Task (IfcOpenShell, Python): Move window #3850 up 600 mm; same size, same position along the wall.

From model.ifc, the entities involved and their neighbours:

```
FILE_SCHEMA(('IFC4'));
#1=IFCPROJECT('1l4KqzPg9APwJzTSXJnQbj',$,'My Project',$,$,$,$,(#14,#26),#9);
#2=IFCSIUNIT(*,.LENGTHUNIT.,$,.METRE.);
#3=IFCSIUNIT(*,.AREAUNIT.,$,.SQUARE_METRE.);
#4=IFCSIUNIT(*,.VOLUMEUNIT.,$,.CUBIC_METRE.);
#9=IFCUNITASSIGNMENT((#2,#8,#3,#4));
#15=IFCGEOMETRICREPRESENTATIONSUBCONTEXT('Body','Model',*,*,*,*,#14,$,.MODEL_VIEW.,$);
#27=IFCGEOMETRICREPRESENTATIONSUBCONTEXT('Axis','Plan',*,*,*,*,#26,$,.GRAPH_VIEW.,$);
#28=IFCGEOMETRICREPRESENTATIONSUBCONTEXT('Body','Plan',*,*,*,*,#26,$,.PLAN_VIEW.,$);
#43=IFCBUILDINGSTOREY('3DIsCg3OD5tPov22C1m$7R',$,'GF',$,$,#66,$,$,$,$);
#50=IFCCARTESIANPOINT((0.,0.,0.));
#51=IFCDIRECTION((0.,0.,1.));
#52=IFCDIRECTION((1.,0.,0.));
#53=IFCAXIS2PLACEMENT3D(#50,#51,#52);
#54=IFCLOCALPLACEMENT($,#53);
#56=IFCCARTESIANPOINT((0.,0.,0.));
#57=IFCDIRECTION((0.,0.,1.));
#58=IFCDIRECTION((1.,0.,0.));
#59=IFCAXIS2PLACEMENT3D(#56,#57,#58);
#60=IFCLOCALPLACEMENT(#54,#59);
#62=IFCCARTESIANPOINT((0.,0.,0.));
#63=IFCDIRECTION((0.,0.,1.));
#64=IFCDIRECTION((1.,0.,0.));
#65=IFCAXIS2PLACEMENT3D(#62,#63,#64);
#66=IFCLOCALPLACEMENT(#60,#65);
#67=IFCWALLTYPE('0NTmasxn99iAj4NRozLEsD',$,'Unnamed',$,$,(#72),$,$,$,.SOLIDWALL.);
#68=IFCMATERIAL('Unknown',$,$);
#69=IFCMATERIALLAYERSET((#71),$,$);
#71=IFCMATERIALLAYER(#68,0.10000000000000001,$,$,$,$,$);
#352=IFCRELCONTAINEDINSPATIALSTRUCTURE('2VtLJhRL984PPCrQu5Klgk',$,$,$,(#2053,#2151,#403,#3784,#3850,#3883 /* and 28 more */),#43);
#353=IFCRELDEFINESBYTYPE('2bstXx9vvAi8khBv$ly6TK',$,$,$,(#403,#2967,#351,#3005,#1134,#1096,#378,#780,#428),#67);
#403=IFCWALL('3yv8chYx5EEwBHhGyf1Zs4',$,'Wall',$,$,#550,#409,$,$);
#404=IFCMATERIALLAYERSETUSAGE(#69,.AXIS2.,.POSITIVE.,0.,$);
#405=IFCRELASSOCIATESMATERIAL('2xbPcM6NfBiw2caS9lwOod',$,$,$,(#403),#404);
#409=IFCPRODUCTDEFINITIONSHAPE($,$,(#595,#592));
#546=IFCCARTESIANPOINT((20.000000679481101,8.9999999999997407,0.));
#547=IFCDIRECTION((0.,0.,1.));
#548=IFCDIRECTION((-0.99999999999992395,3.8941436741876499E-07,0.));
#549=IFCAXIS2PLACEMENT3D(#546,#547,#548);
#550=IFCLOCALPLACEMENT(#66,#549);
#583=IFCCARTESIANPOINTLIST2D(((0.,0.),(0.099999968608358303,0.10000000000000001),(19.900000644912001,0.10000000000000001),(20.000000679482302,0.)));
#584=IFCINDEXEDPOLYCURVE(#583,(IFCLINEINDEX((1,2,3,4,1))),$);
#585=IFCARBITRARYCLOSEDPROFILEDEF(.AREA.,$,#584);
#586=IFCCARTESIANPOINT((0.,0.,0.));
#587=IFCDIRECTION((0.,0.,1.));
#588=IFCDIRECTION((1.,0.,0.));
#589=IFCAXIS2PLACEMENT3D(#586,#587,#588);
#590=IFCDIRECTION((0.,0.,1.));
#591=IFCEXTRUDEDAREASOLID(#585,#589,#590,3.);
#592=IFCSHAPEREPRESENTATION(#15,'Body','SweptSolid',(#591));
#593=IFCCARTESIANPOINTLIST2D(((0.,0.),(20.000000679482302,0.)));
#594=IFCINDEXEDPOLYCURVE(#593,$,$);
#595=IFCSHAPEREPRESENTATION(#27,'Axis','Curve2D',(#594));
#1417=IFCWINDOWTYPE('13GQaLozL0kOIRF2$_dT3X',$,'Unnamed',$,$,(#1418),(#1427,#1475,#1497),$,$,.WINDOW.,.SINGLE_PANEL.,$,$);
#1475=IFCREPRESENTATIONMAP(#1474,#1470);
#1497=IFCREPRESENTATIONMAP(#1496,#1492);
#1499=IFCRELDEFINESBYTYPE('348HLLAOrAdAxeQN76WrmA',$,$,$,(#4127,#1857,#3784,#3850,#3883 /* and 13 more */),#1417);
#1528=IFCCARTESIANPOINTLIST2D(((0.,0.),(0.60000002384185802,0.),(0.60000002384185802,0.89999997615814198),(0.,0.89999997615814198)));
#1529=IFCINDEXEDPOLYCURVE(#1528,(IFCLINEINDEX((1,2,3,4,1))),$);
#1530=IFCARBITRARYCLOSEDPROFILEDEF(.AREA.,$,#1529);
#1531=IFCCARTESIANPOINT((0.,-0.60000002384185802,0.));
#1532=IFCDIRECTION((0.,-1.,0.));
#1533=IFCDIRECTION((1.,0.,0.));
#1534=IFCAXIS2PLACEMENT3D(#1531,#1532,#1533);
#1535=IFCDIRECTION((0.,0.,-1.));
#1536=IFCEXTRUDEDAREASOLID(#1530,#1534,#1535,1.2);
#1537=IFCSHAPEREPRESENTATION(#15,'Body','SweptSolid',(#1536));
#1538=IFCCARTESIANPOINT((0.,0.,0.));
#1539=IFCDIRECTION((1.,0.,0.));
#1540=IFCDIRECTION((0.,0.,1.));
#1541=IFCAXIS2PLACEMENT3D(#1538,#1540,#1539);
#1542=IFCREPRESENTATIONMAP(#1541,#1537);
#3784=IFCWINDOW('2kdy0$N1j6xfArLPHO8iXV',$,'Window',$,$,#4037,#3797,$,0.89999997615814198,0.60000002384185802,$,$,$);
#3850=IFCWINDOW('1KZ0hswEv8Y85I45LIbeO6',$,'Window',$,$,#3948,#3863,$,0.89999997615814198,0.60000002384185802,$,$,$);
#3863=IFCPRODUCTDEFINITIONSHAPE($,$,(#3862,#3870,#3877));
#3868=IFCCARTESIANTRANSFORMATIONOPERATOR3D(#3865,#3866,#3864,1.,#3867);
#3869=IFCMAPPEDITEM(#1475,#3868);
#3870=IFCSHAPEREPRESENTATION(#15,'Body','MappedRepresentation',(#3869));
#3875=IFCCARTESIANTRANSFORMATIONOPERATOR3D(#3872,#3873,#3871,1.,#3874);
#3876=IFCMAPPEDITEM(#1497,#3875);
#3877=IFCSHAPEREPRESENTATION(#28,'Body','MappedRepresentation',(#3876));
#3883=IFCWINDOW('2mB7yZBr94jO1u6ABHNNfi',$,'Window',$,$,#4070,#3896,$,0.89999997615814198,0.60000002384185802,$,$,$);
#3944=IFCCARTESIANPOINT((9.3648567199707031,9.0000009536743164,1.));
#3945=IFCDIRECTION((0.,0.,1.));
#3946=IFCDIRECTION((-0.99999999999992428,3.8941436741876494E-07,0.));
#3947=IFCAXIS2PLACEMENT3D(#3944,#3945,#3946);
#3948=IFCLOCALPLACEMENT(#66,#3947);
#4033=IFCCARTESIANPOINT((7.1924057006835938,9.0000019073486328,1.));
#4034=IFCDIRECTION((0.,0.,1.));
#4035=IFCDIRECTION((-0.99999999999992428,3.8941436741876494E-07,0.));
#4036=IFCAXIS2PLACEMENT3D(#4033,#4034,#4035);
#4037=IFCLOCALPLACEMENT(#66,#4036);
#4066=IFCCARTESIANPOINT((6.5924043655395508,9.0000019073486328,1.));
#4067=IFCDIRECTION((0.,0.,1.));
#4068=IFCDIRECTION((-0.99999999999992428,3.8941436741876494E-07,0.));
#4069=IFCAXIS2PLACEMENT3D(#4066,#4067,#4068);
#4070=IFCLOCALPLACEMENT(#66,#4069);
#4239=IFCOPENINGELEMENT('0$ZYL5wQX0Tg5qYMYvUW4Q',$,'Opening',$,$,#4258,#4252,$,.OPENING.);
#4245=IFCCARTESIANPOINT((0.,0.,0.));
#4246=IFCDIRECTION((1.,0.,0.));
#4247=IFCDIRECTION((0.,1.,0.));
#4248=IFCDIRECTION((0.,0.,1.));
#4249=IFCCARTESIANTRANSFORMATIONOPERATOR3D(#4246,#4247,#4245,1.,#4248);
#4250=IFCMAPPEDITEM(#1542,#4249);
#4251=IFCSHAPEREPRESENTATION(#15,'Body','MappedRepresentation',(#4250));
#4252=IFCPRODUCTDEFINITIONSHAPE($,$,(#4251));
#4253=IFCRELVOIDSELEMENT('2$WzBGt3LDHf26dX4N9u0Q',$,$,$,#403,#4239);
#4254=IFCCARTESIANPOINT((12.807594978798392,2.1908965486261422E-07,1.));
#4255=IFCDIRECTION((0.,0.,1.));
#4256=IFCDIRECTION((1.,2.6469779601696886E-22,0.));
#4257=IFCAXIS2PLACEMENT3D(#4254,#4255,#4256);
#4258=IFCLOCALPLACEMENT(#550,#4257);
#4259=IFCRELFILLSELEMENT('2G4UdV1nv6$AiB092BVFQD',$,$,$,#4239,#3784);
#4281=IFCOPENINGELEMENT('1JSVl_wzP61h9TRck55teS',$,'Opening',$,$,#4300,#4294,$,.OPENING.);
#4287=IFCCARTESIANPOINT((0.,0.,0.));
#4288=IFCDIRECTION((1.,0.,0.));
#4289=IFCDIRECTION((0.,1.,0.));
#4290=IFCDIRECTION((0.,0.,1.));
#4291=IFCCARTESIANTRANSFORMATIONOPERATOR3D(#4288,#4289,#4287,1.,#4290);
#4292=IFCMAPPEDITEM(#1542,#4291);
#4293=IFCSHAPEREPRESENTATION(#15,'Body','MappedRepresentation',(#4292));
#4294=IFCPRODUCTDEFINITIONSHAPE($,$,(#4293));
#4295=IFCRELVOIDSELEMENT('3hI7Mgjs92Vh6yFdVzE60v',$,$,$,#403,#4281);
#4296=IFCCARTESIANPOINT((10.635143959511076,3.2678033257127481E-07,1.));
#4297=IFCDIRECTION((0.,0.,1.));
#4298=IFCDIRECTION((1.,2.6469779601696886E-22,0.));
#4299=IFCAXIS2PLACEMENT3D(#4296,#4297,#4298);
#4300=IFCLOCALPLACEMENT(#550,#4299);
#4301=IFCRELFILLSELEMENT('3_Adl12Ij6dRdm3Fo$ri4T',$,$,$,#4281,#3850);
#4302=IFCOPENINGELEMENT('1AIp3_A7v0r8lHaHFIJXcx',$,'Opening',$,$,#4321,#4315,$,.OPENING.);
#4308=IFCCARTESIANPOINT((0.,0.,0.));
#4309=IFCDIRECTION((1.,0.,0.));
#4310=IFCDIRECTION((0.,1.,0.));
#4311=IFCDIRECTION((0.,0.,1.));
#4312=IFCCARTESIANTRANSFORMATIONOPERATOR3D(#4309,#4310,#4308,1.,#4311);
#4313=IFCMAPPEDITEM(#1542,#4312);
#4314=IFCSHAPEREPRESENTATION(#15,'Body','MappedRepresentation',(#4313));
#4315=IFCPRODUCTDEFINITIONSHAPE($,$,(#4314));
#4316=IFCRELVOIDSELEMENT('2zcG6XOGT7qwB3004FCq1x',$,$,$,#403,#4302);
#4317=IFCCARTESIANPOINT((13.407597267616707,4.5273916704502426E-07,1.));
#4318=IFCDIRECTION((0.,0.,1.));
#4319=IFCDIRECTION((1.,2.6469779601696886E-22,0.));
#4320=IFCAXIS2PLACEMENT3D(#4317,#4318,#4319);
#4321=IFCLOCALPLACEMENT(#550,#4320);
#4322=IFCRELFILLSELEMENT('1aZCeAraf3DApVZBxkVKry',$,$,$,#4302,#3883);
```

```python
import numpy as np
import ifcopenshell
import ifcopenshell.api.geometry
import ifcopenshell.util.placement
import ifcopenshell.util.unit

model = ifcopenshell.open("model.ifc")
unit_scale = ifcopenshell.util.unit.calculate_unit_scale(model)

window = model.by_id(3850)
opening = window.FillsVoids[0].RelatingOpeningElement
dz = 0.6 / unit_scale

shift = np.array([0.0, 0.0, dz])
# The window is not placed relative to its opening, so move both.
for product in (opening, window):
    matrix = ifcopenshell.util.placement.get_local_placement(product.ObjectPlacement)
    matrix[:3, 3] += shift
    ifcopenshell.api.geometry.edit_object_placement(model, product=product, matrix=matrix, is_si=False)

print(f"moved by {dz * unit_scale:+.3f} m")

model.write("model_edited.ifc")
```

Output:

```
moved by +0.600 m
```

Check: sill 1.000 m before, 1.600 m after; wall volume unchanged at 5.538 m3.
